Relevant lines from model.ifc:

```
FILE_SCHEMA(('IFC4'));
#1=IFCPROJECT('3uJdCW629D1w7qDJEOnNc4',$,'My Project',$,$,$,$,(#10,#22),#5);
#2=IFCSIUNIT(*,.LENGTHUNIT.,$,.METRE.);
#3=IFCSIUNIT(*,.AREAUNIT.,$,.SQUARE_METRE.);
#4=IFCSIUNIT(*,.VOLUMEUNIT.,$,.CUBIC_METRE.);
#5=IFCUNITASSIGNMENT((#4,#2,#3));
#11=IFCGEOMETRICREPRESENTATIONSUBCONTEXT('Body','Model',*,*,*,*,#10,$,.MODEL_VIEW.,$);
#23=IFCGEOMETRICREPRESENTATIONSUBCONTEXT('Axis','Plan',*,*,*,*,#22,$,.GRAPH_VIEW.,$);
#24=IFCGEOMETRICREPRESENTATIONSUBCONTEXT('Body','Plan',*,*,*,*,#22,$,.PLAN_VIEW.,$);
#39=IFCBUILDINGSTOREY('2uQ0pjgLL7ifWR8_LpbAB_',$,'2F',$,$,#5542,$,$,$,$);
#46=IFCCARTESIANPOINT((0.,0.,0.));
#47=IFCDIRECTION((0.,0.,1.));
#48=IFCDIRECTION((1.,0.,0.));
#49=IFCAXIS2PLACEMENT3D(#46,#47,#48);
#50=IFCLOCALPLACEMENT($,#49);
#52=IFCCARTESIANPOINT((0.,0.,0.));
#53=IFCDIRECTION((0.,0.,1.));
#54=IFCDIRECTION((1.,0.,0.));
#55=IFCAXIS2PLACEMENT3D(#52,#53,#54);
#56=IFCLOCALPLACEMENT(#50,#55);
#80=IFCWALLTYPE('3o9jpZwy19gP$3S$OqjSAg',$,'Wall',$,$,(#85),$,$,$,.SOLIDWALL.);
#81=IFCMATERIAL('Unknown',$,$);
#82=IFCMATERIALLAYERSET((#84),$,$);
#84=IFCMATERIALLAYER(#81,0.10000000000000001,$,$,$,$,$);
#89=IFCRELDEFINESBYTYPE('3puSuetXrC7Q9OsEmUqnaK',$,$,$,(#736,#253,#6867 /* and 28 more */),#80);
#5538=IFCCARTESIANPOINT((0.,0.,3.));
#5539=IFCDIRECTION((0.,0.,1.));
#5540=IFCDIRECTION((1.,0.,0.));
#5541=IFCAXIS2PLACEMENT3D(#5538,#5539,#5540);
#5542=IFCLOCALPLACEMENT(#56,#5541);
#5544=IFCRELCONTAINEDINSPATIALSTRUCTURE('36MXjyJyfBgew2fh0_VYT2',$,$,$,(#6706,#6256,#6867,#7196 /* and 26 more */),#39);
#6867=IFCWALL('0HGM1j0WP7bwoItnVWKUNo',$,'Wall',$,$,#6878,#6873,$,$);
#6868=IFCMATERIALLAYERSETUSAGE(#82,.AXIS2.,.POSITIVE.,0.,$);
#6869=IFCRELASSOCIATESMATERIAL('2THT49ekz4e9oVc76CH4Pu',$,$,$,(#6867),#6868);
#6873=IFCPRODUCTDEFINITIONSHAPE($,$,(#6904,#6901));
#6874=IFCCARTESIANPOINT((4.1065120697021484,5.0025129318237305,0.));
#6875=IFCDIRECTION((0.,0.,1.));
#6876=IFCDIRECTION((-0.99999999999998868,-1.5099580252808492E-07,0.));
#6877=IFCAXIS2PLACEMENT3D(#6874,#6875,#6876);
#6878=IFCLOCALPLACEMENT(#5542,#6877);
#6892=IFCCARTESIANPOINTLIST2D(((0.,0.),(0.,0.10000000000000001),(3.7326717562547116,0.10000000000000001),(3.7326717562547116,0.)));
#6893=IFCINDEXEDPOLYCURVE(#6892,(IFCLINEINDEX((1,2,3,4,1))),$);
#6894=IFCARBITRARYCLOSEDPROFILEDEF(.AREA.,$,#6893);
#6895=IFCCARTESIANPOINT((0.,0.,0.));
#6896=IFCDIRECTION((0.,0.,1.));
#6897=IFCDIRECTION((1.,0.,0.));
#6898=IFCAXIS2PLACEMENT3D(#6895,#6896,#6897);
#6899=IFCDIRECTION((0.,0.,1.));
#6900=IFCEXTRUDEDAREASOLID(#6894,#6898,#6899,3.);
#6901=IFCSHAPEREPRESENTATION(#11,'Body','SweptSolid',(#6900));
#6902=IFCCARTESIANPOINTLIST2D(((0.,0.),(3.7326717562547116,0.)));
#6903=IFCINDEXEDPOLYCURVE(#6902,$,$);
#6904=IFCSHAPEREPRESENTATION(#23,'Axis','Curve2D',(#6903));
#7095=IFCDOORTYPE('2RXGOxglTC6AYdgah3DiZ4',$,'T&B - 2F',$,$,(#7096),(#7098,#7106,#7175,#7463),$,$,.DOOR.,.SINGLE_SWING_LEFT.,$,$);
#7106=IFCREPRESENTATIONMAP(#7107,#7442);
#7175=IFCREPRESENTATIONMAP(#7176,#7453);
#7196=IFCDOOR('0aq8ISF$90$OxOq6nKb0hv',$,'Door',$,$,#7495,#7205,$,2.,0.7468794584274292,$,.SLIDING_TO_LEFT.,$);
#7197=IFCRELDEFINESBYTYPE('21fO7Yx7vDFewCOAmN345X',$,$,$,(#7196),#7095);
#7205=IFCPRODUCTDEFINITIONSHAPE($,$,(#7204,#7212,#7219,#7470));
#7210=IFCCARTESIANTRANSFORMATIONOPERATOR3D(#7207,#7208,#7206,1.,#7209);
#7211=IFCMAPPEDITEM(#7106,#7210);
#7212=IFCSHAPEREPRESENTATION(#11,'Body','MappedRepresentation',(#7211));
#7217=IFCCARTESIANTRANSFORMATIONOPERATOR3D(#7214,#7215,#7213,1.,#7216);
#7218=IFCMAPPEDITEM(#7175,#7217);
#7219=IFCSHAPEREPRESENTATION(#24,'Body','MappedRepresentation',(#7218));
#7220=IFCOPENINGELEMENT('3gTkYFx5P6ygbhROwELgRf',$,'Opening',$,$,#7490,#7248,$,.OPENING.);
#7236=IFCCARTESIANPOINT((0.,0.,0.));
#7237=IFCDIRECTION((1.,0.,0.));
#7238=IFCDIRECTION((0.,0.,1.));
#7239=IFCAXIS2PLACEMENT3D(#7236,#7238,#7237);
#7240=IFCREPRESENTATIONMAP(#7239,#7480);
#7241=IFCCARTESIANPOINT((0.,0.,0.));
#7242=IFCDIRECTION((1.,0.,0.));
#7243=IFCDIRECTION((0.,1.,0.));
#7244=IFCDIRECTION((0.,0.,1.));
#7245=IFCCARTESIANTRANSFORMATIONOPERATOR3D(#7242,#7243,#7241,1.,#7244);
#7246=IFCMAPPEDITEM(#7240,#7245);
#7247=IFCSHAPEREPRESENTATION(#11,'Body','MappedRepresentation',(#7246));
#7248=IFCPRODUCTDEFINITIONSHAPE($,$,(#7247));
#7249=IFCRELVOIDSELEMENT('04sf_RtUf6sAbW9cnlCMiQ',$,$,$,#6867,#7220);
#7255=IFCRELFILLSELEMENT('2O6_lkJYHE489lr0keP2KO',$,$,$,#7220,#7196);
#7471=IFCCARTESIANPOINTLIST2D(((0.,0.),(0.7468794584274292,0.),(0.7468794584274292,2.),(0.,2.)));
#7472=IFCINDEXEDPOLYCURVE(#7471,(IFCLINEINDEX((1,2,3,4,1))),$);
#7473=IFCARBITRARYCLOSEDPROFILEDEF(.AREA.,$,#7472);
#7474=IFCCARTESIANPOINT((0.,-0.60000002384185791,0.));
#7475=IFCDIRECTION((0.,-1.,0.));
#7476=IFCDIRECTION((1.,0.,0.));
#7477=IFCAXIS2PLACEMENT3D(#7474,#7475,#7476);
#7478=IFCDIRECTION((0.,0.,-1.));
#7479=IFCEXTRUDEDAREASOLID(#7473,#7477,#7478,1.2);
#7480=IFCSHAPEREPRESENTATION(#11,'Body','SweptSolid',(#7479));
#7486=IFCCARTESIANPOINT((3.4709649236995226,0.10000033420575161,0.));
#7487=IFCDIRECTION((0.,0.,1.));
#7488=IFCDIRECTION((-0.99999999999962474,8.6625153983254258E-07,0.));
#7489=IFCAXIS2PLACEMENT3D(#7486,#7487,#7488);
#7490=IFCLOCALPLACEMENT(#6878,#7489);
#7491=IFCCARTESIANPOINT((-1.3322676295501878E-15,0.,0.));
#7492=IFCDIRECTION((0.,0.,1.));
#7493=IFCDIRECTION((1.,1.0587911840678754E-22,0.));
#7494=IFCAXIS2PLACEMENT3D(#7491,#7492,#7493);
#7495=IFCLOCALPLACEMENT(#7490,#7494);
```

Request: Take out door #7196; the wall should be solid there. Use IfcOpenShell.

```python
import ifcopenshell
import ifcopenshell.api.feature
import ifcopenshell.api.root
import ifcopenshell.geom
import ifcopenshell.util.shape

model = ifcopenshell.open("model.ifc")
settings = ifcopenshell.geom.settings()


def volume(element):
    """Net volume in cubic metres, openings subtracted."""
    shape = ifcopenshell.geom.create_shape(settings, element)
    return ifcopenshell.util.shape.get_volume(shape.geometry)


door = model.by_guid("0aq8ISF$90$OxOq6nKb0hv")
opening = door.FillsVoids[0].RelatingOpeningElement
wall = opening.VoidsElements[0].RelatingBuildingElement
before = volume(wall)

ifcopenshell.api.root.remove_product(model, product=door)
ifcopenshell.api.feature.remove_feature(model, feature=opening)

after = volume(wall)

print(f"wall volume {before:.3f} -> {after:.3f} m3")

model.write("model_updated.ifc")
```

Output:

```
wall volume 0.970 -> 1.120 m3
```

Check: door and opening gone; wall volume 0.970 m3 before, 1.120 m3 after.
